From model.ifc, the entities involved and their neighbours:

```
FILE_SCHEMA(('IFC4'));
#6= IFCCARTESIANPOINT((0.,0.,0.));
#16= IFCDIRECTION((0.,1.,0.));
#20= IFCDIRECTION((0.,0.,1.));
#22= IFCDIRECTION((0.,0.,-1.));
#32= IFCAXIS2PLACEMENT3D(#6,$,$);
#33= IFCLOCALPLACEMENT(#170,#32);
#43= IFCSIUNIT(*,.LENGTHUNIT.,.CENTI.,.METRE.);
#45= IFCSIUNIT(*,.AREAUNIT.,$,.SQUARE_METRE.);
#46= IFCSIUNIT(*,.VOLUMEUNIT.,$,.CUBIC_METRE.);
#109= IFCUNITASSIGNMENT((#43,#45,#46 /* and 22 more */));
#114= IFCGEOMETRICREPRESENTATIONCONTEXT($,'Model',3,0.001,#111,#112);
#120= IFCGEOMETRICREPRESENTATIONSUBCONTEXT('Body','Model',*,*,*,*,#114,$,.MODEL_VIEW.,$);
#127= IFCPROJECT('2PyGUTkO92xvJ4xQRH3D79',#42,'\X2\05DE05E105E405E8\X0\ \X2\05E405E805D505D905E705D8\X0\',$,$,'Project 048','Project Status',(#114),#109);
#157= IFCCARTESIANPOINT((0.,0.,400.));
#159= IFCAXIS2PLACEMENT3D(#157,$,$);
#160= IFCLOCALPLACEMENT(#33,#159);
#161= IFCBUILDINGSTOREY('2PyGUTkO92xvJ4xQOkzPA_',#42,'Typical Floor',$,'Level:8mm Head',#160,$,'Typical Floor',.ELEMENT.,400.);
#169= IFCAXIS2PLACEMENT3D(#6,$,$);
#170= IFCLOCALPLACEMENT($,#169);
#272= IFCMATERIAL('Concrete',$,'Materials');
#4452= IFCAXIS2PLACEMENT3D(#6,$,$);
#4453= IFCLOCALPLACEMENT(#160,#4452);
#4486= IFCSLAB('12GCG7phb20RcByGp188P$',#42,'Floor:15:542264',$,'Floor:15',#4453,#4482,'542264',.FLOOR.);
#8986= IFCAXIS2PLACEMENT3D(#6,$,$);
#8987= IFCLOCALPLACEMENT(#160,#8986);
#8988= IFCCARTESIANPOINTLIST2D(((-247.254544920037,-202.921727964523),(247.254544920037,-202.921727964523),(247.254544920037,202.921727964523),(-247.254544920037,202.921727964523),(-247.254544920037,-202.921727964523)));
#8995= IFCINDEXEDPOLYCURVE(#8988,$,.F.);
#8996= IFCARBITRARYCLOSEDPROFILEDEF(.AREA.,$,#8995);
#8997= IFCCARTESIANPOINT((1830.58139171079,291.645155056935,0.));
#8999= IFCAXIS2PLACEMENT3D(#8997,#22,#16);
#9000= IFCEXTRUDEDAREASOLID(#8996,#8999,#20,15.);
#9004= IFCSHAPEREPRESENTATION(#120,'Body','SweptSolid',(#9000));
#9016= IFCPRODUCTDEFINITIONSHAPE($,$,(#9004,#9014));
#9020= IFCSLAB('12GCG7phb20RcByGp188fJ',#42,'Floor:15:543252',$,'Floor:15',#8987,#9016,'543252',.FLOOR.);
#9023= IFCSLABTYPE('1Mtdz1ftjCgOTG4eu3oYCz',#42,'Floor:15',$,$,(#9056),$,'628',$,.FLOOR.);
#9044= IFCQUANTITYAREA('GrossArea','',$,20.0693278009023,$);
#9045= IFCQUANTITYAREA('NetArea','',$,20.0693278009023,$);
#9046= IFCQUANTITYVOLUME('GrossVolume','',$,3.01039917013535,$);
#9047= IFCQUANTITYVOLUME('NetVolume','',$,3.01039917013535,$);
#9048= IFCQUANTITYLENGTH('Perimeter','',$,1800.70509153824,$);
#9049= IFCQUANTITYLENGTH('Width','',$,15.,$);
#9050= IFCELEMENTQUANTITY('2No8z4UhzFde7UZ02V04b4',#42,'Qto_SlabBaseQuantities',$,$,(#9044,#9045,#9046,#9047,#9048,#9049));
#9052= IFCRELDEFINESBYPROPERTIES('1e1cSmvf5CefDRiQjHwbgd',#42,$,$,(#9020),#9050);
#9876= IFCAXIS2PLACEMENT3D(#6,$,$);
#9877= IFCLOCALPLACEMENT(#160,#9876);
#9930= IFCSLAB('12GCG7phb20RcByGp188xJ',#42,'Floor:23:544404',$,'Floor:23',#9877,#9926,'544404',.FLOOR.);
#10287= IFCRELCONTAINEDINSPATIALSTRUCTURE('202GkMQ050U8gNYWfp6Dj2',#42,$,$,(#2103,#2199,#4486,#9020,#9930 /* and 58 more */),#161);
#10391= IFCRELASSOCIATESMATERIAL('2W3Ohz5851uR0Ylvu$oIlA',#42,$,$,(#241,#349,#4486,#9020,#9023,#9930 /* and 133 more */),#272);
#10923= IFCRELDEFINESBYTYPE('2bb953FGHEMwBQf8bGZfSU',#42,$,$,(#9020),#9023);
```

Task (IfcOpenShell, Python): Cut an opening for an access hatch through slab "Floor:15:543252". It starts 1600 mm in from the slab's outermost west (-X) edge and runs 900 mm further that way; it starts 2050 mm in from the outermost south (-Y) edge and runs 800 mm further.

```python
import numpy as np
import ifcopenshell
import ifcopenshell.api.feature
import ifcopenshell.api.geometry
import ifcopenshell.api.pset
import ifcopenshell.api.root
import ifcopenshell.geom
import ifcopenshell.util.element
import ifcopenshell.util.placement
import ifcopenshell.util.representation
import ifcopenshell.util.shape
import ifcopenshell.util.unit

model = ifcopenshell.open("model.ifc")
unit_scale = ifcopenshell.util.unit.calculate_unit_scale(model)
area_scale = ifcopenshell.util.unit.calculate_unit_scale(model, "AREAUNIT")
volume_scale = ifcopenshell.util.unit.calculate_unit_scale(model, "VOLUMEUNIT")
settings = ifcopenshell.geom.settings()


def volume(element):
    """Net volume in cubic metres, openings subtracted."""
    shape = ifcopenshell.geom.create_shape(settings, element)
    return ifcopenshell.util.shape.get_volume(shape.geometry)


slab = model.by_guid("12GCG7phb20RcByGp188fJ")
before = volume(slab)

# Extent in the slab's own axes, in metres. The edges named are its -X and -Y sides.
slab_shape = ifcopenshell.geom.create_shape(settings, slab)
vertices = ifcopenshell.util.shape.get_vertices(slab_shape.geometry)
x_min, y_min, bottom = vertices.min(axis=0)
top = vertices[:, 2].max()

opening = ifcopenshell.api.root.create_entity(model, ifc_class="IfcOpeningElement", name="Access hatch opening", predefined_type="OPENING")
context = ifcopenshell.util.representation.get_context(model, "Model", "Body", "MODEL_VIEW")
width, depth = 0.9, 0.8
outline = [(0.0, 0.0), (width, 0.0), (width, depth), (0.0, depth), (0.0, 0.0)]
# Overshoot both faces by 50 mm so the cut is clean.
shape = ifcopenshell.api.geometry.add_slab_representation(
    model, context=context, depth=top - bottom + 0.1, polyline=outline
)
ifcopenshell.api.geometry.assign_representation(model, product=opening, representation=shape)

matrix = ifcopenshell.util.placement.get_local_placement(slab.ObjectPlacement)
matrix[:, 3] = matrix @ np.append(np.array([x_min + 1.6, y_min + 2.05, bottom - 0.05]) / unit_scale, 1.0)
ifcopenshell.api.geometry.edit_object_placement(model, product=opening, matrix=matrix, is_si=False)
ifcopenshell.api.feature.add_feature(model, feature=opening, element=slab)

after = volume(slab)

# Update the slab's stored quantities.
qto = model.by_id(ifcopenshell.util.element.get_pset(slab, "Qto_SlabBaseQuantities", should_inherit=False)["id"])
ifcopenshell.api.pset.edit_qto(model, qto=qto, properties={
    "NetArea": after / (top - bottom) / area_scale,
    "NetVolume": after / volume_scale,
})

print(f"slab volume {before:.3f} -> {after:.3f} m3")

model.write("model-out.ifc")
```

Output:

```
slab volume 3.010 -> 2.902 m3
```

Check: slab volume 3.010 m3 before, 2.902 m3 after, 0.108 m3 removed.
